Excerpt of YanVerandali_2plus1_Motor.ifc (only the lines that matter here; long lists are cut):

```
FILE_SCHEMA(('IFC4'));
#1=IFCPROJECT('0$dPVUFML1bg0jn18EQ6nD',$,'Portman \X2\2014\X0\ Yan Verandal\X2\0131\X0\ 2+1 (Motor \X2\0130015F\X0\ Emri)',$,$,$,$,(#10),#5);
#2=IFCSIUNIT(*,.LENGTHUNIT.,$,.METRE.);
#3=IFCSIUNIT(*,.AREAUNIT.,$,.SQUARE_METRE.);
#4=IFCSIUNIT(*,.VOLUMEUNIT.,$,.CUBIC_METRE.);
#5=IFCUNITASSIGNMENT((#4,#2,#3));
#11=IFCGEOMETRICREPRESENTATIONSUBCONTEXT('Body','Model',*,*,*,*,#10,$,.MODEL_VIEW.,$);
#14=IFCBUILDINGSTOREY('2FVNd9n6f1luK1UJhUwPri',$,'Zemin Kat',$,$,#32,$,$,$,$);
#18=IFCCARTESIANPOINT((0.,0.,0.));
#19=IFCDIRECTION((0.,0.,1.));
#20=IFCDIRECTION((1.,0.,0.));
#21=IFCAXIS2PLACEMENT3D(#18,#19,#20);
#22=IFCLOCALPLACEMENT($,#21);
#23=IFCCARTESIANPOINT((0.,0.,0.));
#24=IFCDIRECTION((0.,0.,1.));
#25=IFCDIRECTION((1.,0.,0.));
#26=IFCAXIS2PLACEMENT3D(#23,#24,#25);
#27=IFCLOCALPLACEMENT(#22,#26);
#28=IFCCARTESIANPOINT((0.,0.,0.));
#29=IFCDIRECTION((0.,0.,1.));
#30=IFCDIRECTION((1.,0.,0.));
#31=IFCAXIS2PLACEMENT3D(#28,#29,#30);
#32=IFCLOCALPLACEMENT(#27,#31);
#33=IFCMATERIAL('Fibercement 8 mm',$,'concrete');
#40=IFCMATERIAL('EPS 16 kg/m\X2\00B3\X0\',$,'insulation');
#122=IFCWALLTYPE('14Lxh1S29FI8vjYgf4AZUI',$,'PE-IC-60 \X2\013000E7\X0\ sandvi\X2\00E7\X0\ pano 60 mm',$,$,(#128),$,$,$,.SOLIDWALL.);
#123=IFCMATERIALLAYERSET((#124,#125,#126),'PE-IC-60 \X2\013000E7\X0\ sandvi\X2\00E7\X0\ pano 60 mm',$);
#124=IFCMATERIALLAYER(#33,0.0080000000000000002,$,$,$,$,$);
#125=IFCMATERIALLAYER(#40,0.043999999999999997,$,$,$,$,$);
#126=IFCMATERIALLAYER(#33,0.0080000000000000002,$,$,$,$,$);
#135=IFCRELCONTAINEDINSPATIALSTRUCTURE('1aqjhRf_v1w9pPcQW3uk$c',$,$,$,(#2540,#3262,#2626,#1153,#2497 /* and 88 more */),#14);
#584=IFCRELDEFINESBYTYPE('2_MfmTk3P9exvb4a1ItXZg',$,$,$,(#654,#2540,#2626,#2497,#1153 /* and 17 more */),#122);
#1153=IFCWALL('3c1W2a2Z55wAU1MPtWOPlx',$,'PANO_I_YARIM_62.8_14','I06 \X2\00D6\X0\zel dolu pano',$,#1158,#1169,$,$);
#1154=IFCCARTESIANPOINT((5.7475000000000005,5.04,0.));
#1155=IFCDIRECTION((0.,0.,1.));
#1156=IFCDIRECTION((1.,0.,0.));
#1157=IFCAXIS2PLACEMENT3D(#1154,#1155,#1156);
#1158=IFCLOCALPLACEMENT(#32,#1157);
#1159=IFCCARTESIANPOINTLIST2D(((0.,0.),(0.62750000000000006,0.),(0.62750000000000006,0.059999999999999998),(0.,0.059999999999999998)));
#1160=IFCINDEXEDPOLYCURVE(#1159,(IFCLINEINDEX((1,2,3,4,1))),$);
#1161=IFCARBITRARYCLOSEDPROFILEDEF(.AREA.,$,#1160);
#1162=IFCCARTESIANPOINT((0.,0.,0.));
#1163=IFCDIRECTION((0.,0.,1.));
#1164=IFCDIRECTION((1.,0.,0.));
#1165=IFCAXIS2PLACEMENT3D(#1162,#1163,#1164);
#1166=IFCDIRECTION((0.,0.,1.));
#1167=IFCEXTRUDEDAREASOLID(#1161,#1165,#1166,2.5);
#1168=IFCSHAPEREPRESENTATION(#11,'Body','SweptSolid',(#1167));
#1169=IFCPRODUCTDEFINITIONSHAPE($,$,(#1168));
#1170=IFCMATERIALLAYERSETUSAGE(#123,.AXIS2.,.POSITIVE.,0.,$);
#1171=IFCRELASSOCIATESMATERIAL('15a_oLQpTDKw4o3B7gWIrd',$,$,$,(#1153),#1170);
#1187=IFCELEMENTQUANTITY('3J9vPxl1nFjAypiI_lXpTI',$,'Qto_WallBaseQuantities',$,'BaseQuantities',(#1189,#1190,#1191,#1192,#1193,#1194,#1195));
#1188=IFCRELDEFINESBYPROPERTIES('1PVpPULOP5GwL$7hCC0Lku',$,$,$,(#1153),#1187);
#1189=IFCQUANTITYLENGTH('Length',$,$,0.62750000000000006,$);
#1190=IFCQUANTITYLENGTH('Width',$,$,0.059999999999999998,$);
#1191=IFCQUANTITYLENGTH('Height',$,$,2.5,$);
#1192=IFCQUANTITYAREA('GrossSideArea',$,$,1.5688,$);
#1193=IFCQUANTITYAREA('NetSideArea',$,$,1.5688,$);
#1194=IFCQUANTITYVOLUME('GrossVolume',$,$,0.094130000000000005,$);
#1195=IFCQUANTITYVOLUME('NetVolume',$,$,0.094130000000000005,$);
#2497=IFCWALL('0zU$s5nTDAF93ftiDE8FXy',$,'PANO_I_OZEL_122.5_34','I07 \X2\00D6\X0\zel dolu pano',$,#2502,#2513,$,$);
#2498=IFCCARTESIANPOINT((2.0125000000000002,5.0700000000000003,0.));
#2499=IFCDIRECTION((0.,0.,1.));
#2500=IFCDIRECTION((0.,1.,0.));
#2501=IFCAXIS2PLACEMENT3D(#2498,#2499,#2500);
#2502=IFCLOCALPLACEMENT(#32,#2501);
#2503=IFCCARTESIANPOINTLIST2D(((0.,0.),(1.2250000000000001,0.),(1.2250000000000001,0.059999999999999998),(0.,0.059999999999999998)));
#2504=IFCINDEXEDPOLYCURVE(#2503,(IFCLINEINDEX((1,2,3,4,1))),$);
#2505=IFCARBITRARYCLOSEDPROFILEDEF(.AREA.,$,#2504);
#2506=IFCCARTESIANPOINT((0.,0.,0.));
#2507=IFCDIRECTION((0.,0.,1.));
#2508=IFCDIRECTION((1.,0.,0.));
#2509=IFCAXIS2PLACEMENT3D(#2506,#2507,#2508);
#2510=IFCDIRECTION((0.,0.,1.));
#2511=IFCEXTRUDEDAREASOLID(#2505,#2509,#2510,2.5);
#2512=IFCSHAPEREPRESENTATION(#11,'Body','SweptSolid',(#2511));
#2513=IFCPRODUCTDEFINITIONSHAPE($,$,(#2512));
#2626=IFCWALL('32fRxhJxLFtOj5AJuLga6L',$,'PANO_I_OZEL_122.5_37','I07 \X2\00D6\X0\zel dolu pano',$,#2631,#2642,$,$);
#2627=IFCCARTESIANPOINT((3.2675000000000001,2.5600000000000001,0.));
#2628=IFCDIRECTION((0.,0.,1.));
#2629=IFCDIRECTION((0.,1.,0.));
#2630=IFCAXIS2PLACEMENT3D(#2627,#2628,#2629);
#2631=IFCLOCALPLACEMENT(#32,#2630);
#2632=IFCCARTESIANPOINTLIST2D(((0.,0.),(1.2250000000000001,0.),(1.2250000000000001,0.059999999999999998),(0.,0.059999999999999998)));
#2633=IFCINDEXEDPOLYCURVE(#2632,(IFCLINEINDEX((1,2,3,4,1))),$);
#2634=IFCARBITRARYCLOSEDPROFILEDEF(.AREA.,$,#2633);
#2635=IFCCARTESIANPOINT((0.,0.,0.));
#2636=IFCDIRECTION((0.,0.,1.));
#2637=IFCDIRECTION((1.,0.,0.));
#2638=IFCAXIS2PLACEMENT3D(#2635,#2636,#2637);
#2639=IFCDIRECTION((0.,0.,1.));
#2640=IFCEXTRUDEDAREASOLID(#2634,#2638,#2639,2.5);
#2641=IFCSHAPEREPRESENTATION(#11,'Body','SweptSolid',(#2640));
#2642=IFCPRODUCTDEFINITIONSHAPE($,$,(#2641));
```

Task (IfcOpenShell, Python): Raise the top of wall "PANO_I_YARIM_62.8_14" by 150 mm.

```python
import ifcopenshell
import ifcopenshell.api.pset
import ifcopenshell.geom
import ifcopenshell.util.element
import ifcopenshell.util.representation
import ifcopenshell.util.shape
import ifcopenshell.util.unit

model = ifcopenshell.open("YanVerandali_2plus1_Motor.ifc")
unit_scale = ifcopenshell.util.unit.calculate_unit_scale(model)
area_scale = ifcopenshell.util.unit.calculate_unit_scale(model, "AREAUNIT")
volume_scale = ifcopenshell.util.unit.calculate_unit_scale(model, "VOLUMEUNIT")
settings = ifcopenshell.geom.settings()


def volume(element):
    """Net volume in cubic metres, openings subtracted."""
    shape = ifcopenshell.geom.create_shape(settings, element)
    return ifcopenshell.util.shape.get_volume(shape.geometry)


wall = model.by_guid("3c1W2a2Z55wAU1MPtWOPlx")
before = volume(wall)

body = ifcopenshell.util.representation.get_representation(wall, "Model", "Body")
solid = body.Items[0]
old_height = solid.Depth
solid.Depth += 0.15
after = volume(wall)
thickness = 0.06  # wall thickness in metres

# Update the stored height, areas and volumes.
qto = model.by_id(ifcopenshell.util.element.get_pset(wall, "Qto_WallBaseQuantities", should_inherit=False)["id"])
ifcopenshell.api.pset.edit_qto(model, qto=qto, properties={
    "Height": solid.Depth,
    "GrossSideArea": ifcopenshell.util.element.get_pset(wall, "Qto_WallBaseQuantities", "GrossSideArea") * solid.Depth / old_height,
    "NetSideArea": after / thickness / area_scale,
    "GrossVolume": ifcopenshell.util.element.get_pset(wall, "Qto_WallBaseQuantities", "GrossVolume") * solid.Depth / old_height,
    "NetVolume": after / volume_scale,
})

print(f"height {old_height:g} -> {solid.Depth:g}, volume {before:.3f} -> {after:.3f} m3")

model.write("YanVerandali_2plus1_Motor_rev.ifc")
```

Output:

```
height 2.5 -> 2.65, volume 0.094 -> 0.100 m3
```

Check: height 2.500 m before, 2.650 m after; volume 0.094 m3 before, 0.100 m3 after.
